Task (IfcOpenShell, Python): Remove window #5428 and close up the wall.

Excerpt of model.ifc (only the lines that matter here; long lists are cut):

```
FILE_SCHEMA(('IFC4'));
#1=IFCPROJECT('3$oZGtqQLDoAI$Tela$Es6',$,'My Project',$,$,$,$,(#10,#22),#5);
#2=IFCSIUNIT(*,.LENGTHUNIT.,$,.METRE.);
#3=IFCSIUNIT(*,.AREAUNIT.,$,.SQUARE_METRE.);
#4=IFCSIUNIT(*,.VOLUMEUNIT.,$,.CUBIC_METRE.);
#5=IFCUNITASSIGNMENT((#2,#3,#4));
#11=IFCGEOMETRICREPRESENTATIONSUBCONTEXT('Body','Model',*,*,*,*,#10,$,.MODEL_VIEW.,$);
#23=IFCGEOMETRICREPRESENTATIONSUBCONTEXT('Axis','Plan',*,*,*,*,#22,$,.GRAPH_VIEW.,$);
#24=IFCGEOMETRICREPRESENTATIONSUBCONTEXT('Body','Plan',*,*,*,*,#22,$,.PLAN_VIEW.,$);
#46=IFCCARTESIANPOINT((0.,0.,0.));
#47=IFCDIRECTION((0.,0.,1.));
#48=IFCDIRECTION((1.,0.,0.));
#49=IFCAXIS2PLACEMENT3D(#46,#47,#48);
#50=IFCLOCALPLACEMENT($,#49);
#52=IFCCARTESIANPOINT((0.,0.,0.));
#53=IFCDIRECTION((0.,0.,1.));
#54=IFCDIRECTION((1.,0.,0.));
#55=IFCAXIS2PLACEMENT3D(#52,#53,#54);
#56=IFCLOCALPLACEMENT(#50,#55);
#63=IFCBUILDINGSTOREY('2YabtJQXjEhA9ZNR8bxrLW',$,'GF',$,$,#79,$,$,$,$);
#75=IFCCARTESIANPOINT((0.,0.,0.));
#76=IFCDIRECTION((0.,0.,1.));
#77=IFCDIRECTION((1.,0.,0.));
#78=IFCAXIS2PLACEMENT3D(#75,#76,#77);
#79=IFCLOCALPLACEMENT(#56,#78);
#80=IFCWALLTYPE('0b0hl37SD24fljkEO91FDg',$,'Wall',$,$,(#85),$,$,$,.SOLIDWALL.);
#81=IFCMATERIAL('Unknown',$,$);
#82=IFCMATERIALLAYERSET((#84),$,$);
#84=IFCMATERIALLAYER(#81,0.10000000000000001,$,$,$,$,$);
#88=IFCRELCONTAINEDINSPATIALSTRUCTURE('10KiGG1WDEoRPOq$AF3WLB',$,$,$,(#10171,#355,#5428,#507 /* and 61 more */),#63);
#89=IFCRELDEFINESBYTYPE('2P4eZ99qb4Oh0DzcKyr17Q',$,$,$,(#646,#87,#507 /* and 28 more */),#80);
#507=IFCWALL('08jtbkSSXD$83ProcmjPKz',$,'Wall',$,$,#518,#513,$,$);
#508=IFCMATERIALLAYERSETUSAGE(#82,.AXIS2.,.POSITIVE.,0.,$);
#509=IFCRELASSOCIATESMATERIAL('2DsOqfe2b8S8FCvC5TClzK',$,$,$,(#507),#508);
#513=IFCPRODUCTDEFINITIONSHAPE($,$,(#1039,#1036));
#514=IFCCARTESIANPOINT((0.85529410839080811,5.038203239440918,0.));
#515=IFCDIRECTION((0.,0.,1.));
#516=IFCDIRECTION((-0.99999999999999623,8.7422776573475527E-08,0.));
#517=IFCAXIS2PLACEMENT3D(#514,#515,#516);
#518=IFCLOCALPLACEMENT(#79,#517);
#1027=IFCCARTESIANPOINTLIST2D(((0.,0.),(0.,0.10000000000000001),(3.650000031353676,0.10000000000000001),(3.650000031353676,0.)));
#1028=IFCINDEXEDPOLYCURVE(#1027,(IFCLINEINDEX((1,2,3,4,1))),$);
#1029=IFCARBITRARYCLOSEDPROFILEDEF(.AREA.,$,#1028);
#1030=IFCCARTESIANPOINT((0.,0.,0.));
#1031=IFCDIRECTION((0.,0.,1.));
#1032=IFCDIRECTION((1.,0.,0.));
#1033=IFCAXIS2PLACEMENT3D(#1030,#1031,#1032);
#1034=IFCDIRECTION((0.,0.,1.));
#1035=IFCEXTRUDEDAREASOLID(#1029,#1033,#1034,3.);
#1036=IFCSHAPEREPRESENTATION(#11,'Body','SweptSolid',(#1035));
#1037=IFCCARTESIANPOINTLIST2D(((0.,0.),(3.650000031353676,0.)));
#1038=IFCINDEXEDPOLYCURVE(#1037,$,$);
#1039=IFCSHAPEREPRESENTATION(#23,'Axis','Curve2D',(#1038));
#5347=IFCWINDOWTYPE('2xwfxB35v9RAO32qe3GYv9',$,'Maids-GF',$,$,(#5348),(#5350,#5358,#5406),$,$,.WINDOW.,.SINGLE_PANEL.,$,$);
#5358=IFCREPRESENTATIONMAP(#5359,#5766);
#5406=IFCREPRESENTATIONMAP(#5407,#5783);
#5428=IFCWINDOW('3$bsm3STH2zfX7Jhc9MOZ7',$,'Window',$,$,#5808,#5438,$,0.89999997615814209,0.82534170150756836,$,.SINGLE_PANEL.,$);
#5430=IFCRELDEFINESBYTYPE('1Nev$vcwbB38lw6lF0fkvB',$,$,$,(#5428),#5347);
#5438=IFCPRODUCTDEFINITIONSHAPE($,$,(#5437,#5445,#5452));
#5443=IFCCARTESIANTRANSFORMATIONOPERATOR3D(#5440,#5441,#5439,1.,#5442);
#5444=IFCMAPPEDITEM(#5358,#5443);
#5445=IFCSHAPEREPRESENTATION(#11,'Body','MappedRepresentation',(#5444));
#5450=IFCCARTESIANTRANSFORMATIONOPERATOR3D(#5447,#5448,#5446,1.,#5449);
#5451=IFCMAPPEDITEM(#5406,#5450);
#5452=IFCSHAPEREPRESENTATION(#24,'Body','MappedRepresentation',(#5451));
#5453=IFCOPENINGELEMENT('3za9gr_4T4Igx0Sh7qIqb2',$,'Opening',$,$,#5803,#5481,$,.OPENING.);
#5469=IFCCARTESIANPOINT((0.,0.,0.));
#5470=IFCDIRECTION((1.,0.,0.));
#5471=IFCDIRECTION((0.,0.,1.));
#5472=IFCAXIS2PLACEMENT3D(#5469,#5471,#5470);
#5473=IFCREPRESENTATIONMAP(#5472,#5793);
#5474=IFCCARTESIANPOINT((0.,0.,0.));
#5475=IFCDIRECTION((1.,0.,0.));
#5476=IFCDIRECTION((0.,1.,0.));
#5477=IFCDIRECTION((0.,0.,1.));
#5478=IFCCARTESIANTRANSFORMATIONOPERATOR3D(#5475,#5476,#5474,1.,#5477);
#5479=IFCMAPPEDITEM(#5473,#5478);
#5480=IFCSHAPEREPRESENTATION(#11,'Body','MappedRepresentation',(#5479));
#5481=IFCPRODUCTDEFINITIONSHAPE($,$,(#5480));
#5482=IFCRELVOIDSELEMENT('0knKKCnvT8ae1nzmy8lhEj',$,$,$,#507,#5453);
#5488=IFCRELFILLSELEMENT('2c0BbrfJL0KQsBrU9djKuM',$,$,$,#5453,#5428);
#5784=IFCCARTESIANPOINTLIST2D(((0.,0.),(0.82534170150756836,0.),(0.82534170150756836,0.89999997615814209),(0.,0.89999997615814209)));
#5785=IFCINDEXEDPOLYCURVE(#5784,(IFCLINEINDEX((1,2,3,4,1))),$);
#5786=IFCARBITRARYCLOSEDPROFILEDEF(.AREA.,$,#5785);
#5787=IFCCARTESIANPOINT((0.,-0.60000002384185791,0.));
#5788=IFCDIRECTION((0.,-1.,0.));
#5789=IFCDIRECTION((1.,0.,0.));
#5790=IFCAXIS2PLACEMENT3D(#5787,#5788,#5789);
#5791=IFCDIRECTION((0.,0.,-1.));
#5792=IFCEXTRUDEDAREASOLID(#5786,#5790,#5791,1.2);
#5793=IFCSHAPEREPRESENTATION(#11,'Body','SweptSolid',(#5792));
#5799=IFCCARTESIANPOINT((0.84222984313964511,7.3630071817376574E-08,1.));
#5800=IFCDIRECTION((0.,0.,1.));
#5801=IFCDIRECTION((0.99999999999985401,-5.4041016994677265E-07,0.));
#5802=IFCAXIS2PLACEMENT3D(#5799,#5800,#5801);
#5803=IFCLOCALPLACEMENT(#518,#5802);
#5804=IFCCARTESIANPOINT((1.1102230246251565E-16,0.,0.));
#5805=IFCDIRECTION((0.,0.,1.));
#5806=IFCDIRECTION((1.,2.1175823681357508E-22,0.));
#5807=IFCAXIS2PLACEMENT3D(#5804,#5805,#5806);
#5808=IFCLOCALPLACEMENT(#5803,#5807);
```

```python
import ifcopenshell
import ifcopenshell.api.feature
import ifcopenshell.api.root
import ifcopenshell.geom
import ifcopenshell.util.shape

model = ifcopenshell.open("model.ifc")
settings = ifcopenshell.geom.settings()


def volume(element):
    """Net volume in cubic metres, openings subtracted."""
    shape = ifcopenshell.geom.create_shape(settings, element)
    return ifcopenshell.util.shape.get_volume(shape.geometry)


window = model.by_guid("3$bsm3STH2zfX7Jhc9MOZ7")
opening = window.FillsVoids[0].RelatingOpeningElement
wall = opening.VoidsElements[0].RelatingBuildingElement
before = volume(wall)

ifcopenshell.api.root.remove_product(model, product=window)
ifcopenshell.api.feature.remove_feature(model, feature=opening)

after = volume(wall)

print(f"wall volume {before:.3f} -> {after:.3f} m3")

model.write("model-out.ifc")
```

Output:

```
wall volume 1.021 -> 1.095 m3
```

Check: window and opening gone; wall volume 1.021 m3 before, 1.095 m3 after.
